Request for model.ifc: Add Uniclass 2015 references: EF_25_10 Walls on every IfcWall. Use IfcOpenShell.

First a look at what the model holds.

```python
import ifcopenshell

model = ifcopenshell.open("model.ifc")
print(model.schema)
print("classifications:", [c.Name for c in model.by_type("IfcClassification")])
for ifc_class in ("IfcDoor", "IfcRoof", "IfcStair", "IfcWall", "IfcWindow"):
    print(ifc_class, len(model.by_type(ifc_class)))
```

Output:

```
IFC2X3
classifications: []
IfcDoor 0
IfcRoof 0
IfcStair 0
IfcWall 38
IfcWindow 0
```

```python
import ifcopenshell
import ifcopenshell.api.classification

model = ifcopenshell.open("model.ifc")

# IFC2X3 requires Source and Edition and has no link from the project to the system.
system = model.create_entity("IfcClassification", Source="NBS", Edition="2015", Name="Uniclass 2015")

codes = {
    "IfcWall": ("EF_25_10", "Walls"),
}
for ifc_class, (code, name) in codes.items():
    products = model.by_type(ifc_class)
    ifcopenshell.api.classification.add_reference(
        model, products=products, classification=system, identification=code, name=name
    )
    print(code, len(products))

model.write("model-out.ifc")
```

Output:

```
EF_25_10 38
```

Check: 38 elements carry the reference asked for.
